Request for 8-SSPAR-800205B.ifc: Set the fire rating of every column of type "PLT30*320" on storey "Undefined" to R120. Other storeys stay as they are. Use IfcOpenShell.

First a look at what the model holds.

```python
import ifcopenshell
import ifcopenshell.util.element

model = ifcopenshell.open("8-SSPAR-800205B.ifc")
print(model.schema)
storey = next(s for s in model.by_type("IfcBuildingStorey") if s.Name == "Undefined")
columns = [e for e in ifcopenshell.util.element.get_decomposition(storey) if e.is_a("IfcColumn")]
seen = {}
for e in columns:
    element_type = ifcopenshell.util.element.get_type(e)
    key = (element_type.Name if element_type != e and element_type else None, ifcopenshell.util.element.get_pset(e, "Pset_ColumnCommon", "FireRating"))
    seen[key] = seen.get(key, 0) + 1
for (name, value), count in sorted(seen.items(), key=str):
    print(count, "x", name, "|", value)
```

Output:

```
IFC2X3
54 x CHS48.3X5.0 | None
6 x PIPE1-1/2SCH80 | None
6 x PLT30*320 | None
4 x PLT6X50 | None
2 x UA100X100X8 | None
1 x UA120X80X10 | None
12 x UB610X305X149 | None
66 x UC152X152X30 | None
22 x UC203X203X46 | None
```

```python
import ifcopenshell
import ifcopenshell.api.pset
import ifcopenshell.util.element

model = ifcopenshell.open("8-SSPAR-800205B.ifc")

storey = next(s for s in model.by_type("IfcBuildingStorey") if s.Name == "Undefined")
columns = [e for e in ifcopenshell.util.element.get_decomposition(storey) if e.is_a("IfcColumn")]

count = 0
for e in columns:
    element_type = ifcopenshell.util.element.get_type(e)
    if element_type in (None, e) or element_type.Name != "PLT30*320":
        continue
    # add_pset returns the element's existing set when there is one.
    pset = ifcopenshell.api.pset.add_pset(model, product=e, name="Pset_ColumnCommon")
    ifcopenshell.api.pset.edit_pset(model, pset=pset, properties={"FireRating": "R120"})
    count += 1

print(count, "columns updated")

model.write("8-SSPAR-800205B_rev.ifc")
```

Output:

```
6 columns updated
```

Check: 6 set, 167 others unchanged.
